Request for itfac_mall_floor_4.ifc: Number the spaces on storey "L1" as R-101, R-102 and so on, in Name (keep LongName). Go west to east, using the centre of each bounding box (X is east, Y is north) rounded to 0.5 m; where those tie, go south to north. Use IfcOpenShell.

First a look at what the model holds.

```python
import ifcopenshell
import ifcopenshell.util.element
import ifcopenshell.util.placement

model = ifcopenshell.open("itfac_mall_floor_4.ifc")
print(model.schema)
storey = next(s for s in model.by_type("IfcBuildingStorey") if s.Name == "L1")
spaces = [e for e in ifcopenshell.util.element.get_decomposition(storey) if e.is_a("IfcSpace")]
for e in sorted(spaces, key=lambda e: e.id()):
    origin = ifcopenshell.util.placement.get_local_placement(e.ObjectPlacement)[:3, 3]
    print(e.id(), e.Name, e.LongName, origin.round(2) + 0.0, sep=" | ")
```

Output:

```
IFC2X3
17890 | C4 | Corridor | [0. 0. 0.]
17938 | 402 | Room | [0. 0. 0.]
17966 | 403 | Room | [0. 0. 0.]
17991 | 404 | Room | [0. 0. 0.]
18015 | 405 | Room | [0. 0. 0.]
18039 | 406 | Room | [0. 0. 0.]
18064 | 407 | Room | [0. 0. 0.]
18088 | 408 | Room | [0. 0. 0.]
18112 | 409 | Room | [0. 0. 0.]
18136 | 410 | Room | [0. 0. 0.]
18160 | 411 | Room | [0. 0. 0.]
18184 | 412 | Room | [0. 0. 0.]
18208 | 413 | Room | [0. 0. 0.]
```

```python
import ifcopenshell
import ifcopenshell.geom
import ifcopenshell.util.element
import ifcopenshell.util.shape

model = ifcopenshell.open("itfac_mall_floor_4.ifc")
settings = ifcopenshell.geom.settings()
settings.set("use-world-coords", True)


def centre(element):
    shape = ifcopenshell.geom.create_shape(settings, element)
    return ifcopenshell.util.shape.get_bbox_centroid(shape.geometry)


storey = next(s for s in model.by_type("IfcBuildingStorey") if s.Name == "L1")
spaces = [e for e in ifcopenshell.util.element.get_decomposition(storey) if e.is_a("IfcSpace")]

# Insertion points can sit at a corner or the storey origin, so sort by the geometry (in metres).
centres = {e: centre(e) for e in spaces}
spaces.sort(key=lambda e: (round(centres[e][0] / 0.5), centres[e][1]))

for i, e in enumerate(spaces, start=1):
    number = f"R-1{i:02d}"
    e.Name = number
    print(e.id(), number)

model.write("itfac_mall_floor_4_rev.ifc")
```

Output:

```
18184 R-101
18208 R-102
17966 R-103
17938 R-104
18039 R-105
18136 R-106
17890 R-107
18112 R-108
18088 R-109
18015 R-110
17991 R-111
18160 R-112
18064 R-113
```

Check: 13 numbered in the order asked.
